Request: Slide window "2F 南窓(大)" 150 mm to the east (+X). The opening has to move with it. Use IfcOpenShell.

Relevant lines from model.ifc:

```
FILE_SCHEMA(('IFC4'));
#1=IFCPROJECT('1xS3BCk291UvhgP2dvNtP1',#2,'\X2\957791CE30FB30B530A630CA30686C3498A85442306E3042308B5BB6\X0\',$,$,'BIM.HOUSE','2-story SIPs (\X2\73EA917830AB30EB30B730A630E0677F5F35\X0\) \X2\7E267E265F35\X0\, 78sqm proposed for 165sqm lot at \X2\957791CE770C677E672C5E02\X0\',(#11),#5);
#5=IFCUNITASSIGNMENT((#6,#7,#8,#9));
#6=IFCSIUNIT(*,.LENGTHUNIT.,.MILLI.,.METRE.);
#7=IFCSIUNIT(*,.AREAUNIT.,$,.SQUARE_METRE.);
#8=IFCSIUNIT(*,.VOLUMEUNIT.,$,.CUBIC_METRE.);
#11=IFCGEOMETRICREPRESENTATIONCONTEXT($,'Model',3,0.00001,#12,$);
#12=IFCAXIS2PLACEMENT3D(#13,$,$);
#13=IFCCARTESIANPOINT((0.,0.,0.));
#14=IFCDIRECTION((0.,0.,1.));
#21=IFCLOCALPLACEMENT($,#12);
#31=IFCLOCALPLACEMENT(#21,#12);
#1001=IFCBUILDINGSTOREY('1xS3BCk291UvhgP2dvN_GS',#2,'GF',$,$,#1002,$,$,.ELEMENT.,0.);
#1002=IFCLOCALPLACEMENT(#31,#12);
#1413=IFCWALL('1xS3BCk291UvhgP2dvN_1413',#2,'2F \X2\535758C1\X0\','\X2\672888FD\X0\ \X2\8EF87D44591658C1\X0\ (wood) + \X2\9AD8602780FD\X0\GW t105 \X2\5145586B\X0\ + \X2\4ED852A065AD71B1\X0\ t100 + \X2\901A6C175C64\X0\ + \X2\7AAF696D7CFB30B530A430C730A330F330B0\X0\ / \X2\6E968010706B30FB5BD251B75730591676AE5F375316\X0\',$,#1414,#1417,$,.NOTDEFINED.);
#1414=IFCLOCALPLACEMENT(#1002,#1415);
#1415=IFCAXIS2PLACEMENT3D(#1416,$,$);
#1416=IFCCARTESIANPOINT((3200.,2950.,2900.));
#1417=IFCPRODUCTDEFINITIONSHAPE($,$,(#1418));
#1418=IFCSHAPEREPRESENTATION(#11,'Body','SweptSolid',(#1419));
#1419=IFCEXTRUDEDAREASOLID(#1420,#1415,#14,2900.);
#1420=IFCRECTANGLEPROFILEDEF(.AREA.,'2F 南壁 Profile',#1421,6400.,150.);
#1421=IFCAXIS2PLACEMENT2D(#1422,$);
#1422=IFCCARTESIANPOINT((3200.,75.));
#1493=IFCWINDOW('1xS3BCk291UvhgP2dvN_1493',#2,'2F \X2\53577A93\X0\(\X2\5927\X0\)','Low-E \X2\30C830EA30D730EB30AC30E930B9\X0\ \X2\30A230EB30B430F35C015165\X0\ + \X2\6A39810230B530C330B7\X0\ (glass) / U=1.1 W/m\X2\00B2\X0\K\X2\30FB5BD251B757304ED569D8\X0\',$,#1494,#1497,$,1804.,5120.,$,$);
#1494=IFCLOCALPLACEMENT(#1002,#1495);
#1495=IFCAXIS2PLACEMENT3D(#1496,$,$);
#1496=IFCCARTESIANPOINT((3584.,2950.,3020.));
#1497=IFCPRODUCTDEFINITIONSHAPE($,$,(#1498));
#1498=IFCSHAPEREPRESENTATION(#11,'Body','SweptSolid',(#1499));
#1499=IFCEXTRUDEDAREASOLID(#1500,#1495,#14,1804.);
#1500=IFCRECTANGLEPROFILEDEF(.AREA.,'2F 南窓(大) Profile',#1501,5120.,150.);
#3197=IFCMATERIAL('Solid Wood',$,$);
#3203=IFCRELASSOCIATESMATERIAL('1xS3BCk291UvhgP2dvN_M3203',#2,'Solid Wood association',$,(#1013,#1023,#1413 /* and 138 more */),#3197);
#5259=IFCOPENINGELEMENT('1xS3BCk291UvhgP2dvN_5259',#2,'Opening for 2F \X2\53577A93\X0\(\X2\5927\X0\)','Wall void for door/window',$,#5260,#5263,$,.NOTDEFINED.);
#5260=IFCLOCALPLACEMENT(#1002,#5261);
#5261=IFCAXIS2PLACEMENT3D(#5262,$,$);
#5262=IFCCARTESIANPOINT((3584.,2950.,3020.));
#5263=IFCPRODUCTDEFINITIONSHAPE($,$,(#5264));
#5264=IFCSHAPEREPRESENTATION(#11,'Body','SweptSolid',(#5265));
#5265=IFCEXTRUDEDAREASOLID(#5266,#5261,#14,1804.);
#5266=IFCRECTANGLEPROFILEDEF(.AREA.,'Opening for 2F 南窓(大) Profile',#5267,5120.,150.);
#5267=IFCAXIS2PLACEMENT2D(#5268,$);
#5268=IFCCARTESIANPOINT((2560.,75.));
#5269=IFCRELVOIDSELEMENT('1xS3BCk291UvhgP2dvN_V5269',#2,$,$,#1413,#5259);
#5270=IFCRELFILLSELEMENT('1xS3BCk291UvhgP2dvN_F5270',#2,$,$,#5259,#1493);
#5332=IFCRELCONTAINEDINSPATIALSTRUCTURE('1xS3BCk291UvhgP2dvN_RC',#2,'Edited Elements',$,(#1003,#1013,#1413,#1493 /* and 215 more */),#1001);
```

```python
import ifcopenshell
import ifcopenshell.api.geometry
import ifcopenshell.util.placement

model = ifcopenshell.open("model.ifc")

window = model.by_guid("1xS3BCk291UvhgP2dvN_1493")
opening = window.FillsVoids[0].RelatingOpeningElement
wall = opening.VoidsElements[0].RelatingBuildingElement

wall_matrix = ifcopenshell.util.placement.get_local_placement(wall.ObjectPlacement)
shift = wall_matrix[:3, 0] * 150.0
before = ifcopenshell.util.placement.get_local_placement(window.ObjectPlacement)[:3, 3].copy()

# The window is not placed relative to its opening, so move both.
for product in (opening, window):
    matrix = ifcopenshell.util.placement.get_local_placement(product.ObjectPlacement)
    matrix[:3, 3] += shift
    ifcopenshell.api.geometry.edit_object_placement(model, product=product, matrix=matrix, is_si=False)

after = ifcopenshell.util.placement.get_local_placement(window.ObjectPlacement)[:3, 3]
print("window moved by", (after - before).round(3) + 0.0)

model.write("model_rev.ifc")
```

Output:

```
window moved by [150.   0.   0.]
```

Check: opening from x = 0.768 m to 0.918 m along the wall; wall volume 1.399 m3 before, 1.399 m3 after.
